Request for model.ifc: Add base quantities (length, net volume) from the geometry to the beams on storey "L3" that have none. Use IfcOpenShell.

First a look at what the model holds.

```python
import ifcopenshell
import ifcopenshell.util.element
import ifcopenshell.util.unit

model = ifcopenshell.open("model.ifc")
print(model.schema)
for unit_type in ("LENGTHUNIT", "AREAUNIT", "VOLUMEUNIT"):
    print(unit_type, ifcopenshell.util.unit.calculate_unit_scale(model, unit_type))
storey = next(s for s in model.by_type("IfcBuildingStorey") if s.Name == "L3")
beams = [e for e in ifcopenshell.util.element.get_decomposition(storey) if e.is_a("IfcBeam")]
for e in sorted(beams, key=lambda e: e.id()):
    print(e.id(), e.is_a(), e.Name, list(ifcopenshell.util.element.get_psets(e, qtos_only=True)), sep=" | ")
```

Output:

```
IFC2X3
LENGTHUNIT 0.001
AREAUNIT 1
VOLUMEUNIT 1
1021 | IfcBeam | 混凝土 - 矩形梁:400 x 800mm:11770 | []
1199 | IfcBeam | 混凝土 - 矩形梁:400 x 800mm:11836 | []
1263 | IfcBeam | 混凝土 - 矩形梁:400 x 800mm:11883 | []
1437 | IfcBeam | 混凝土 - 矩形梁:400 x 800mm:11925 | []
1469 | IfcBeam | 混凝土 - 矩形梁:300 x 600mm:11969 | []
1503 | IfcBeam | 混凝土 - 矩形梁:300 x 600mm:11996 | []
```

```python
import ifcopenshell
import ifcopenshell.api.pset
import ifcopenshell.geom
import ifcopenshell.util.element
import ifcopenshell.util.shape
import ifcopenshell.util.unit

model = ifcopenshell.open("model.ifc")
unit_scale = ifcopenshell.util.unit.calculate_unit_scale(model)
volume_scale = ifcopenshell.util.unit.calculate_unit_scale(model, "VOLUMEUNIT")
settings = ifcopenshell.geom.settings()

storey = next(s for s in model.by_type("IfcBuildingStorey") if s.Name == "L3")
beams = [e for e in ifcopenshell.util.element.get_decomposition(storey) if e.is_a("IfcBeam")]

for e in sorted(beams, key=lambda e: e.id()):
    if ifcopenshell.util.element.get_psets(e, qtos_only=True, should_inherit=False):
        continue
    # Geometry comes back in metres, in the element's own axes.
    shape = ifcopenshell.geom.create_shape(settings, e)
    values = {
        "Length": ifcopenshell.util.shape.get_max_xyz(shape.geometry) / unit_scale,
        "NetVolume": ifcopenshell.util.shape.get_volume(shape.geometry) / volume_scale,
    }
    qto = ifcopenshell.api.pset.add_qto(model, product=e, name="BaseQuantities")
    ifcopenshell.api.pset.edit_qto(model, qto=qto, properties=values)
    print(e.id(), {k: round(v, 3) for k, v in values.items()})

model.write("model_v2.ifc")
```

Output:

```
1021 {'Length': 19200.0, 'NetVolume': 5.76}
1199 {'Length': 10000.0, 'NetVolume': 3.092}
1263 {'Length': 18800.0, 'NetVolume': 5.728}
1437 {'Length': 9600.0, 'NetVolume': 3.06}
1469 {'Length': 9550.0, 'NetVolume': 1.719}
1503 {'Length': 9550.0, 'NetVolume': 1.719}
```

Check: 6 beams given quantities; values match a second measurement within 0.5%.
